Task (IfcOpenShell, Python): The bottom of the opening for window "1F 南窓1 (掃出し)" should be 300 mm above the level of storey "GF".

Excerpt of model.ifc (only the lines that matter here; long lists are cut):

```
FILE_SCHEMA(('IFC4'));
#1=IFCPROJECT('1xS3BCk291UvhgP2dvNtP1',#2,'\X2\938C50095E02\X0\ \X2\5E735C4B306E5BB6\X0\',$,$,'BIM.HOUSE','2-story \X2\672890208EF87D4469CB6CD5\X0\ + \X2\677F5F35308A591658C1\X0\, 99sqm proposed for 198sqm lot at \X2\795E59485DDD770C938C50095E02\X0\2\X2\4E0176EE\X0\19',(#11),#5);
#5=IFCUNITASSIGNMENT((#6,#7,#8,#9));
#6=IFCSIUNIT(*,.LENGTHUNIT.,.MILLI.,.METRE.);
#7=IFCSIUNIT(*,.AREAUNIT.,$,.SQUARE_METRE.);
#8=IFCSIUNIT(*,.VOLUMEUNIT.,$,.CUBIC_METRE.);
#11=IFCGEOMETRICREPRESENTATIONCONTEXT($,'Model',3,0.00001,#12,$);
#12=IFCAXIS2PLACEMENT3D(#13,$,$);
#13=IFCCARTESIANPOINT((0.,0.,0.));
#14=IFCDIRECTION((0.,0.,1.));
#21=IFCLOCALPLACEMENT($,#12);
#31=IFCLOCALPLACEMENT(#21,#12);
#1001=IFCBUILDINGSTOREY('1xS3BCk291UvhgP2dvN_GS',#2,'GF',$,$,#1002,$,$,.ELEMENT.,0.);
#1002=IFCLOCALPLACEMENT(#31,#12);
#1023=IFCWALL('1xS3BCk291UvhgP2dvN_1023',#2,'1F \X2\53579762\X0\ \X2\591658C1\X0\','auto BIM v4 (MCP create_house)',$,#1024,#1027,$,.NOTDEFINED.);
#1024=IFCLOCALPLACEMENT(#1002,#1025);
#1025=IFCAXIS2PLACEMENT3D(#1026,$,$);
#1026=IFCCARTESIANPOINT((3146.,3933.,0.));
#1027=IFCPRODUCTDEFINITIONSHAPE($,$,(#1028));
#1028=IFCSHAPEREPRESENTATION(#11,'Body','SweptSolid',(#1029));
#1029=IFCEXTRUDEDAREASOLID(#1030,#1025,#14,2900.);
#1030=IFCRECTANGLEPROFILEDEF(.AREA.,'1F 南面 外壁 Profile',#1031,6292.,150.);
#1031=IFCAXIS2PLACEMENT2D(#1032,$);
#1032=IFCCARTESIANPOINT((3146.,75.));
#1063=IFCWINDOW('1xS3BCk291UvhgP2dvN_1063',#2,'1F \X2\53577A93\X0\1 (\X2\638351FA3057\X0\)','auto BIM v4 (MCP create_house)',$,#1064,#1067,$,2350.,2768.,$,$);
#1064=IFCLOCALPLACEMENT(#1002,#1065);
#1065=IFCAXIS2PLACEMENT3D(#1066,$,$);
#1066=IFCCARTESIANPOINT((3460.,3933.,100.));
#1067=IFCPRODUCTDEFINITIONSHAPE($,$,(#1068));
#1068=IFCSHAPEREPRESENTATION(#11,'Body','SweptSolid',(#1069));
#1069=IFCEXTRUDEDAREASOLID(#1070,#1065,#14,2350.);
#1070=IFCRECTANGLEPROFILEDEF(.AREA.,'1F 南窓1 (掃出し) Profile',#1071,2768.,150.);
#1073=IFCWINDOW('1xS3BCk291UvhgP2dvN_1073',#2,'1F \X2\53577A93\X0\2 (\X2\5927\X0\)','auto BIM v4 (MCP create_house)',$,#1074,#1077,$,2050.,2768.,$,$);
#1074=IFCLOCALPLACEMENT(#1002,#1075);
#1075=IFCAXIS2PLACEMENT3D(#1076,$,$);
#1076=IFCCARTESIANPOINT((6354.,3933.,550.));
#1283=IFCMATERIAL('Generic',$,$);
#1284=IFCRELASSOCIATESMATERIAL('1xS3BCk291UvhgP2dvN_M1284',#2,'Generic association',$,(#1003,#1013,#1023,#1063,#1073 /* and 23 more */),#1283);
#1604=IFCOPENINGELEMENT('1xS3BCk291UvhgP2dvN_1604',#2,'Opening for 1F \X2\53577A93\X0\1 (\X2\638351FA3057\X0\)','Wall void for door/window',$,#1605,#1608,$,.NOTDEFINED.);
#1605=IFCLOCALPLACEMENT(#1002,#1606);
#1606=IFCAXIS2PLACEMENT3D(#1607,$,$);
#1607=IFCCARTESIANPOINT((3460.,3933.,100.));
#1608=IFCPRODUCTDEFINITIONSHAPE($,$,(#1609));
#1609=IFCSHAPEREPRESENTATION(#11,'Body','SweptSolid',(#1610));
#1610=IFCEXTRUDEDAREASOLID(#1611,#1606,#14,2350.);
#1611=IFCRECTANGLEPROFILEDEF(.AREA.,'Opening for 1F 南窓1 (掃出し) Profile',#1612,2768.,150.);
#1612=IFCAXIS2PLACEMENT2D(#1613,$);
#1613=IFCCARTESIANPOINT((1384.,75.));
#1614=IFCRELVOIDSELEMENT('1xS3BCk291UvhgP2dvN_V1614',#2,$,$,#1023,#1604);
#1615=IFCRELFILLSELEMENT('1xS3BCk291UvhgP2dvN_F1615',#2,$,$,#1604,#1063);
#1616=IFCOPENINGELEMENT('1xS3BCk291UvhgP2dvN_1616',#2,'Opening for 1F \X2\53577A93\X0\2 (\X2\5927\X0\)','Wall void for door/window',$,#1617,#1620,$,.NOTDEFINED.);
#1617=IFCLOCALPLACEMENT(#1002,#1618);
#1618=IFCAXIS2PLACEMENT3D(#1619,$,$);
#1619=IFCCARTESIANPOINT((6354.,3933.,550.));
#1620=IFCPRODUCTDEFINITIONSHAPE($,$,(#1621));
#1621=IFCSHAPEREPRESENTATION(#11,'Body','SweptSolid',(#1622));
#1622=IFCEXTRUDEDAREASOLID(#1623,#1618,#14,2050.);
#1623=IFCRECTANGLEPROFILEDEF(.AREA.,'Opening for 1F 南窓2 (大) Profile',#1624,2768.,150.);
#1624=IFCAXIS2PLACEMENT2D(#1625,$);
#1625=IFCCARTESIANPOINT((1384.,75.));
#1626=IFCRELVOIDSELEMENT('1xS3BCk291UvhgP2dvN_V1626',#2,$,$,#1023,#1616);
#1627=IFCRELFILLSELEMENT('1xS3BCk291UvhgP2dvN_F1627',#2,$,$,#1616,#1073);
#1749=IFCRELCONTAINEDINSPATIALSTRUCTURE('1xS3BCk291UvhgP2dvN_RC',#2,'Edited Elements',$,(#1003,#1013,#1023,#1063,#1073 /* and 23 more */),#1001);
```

```python
import numpy as np
import ifcopenshell
import ifcopenshell.api.geometry
import ifcopenshell.geom
import ifcopenshell.util.element
import ifcopenshell.util.placement
import ifcopenshell.util.shape
import ifcopenshell.util.unit

model = ifcopenshell.open("model.ifc")
unit_scale = ifcopenshell.util.unit.calculate_unit_scale(model)

window = model.by_id(1063)
opening = window.FillsVoids[0].RelatingOpeningElement
storey = ifcopenshell.util.element.get_container(window, ifc_class="IfcBuildingStorey")
level = ifcopenshell.util.placement.get_local_placement(storey.ObjectPlacement)[2, 3]

# The opening's origin need not be at the sill, so measure its lowest point.
shape = ifcopenshell.geom.create_shape(ifcopenshell.geom.settings(), opening)
bottom = ifcopenshell.util.shape.get_shape_bottom_elevation(shape, shape.geometry) / unit_scale
dz = level + 0.3 / unit_scale - bottom

shift = np.array([0.0, 0.0, dz])
# The window is not placed relative to its opening, so move both.
for product in (opening, window):
    matrix = ifcopenshell.util.placement.get_local_placement(product.ObjectPlacement)
    matrix[:3, 3] += shift
    ifcopenshell.api.geometry.edit_object_placement(model, product=product, matrix=matrix, is_si=False)

print(f"moved by {dz * unit_scale:+.3f} m")

model.write("model_rev.ifc")
```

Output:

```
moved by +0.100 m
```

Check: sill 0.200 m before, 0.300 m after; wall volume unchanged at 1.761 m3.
